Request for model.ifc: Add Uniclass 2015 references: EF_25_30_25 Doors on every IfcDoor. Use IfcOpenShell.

First a look at what the model holds.

```python
import ifcopenshell

model = ifcopenshell.open("model.ifc")
print(model.schema)
print("classifications:", [c.Name for c in model.by_type("IfcClassification")])
for ifc_class in ("IfcDoor", "IfcRoof", "IfcStair", "IfcWall", "IfcWindow"):
    print(ifc_class, len(model.by_type(ifc_class)))
```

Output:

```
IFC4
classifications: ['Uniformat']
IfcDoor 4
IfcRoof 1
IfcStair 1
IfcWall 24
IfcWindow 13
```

```python
import ifcopenshell
import ifcopenshell.api.classification

model = ifcopenshell.open("model.ifc")

system = ifcopenshell.api.classification.add_classification(model, classification="Uniclass 2015")

codes = {
    "IfcDoor": ("EF_25_30_25", "Doors"),
}
for ifc_class, (code, name) in codes.items():
    products = model.by_type(ifc_class)
    ifcopenshell.api.classification.add_reference(
        model, products=products, classification=system, identification=code, name=name
    )
    print(code, len(products))

model.write("model_updated.ifc")
```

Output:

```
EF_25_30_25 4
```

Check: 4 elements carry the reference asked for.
